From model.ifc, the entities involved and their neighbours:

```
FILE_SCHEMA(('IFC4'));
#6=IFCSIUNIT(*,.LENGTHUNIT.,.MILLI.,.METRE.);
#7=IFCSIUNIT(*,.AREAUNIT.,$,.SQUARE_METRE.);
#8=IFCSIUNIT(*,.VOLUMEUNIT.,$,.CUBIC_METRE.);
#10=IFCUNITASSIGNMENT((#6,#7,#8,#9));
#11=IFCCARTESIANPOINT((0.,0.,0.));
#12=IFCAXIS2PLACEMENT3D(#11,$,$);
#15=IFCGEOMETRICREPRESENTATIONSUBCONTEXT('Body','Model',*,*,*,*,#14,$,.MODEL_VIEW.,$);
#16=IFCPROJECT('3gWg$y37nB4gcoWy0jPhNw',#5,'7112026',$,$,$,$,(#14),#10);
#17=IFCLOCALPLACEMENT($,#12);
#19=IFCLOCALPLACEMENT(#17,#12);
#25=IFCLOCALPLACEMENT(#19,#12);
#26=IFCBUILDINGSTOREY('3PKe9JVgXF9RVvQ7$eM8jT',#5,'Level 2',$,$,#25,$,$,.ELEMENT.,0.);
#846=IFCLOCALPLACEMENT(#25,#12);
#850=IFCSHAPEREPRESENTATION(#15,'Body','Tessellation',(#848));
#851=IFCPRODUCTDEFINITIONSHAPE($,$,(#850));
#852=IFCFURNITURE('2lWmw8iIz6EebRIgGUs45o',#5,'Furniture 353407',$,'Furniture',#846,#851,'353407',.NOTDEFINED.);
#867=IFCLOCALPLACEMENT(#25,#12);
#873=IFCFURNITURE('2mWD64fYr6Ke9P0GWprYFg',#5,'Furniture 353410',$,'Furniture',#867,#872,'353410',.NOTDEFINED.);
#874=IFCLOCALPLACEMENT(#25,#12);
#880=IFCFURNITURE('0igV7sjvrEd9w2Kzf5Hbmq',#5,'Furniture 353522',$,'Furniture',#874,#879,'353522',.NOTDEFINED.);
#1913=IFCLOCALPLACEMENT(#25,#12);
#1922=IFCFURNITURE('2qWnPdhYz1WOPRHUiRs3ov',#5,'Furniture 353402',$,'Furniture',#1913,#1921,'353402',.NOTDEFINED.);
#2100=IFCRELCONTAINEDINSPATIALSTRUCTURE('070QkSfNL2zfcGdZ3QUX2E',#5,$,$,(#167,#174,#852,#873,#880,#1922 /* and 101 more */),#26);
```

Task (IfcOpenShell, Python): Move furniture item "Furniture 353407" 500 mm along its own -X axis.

```python
import ifcopenshell
import ifcopenshell.api.geometry
import ifcopenshell.util.placement
import ifcopenshell.util.unit

model = ifcopenshell.open("model.ifc")
unit_scale = ifcopenshell.util.unit.calculate_unit_scale(model)

item = model.by_guid("2lWmw8iIz6EebRIgGUs45o")
matrix = ifcopenshell.util.placement.get_local_placement(item.ObjectPlacement)
matrix[:3, 3] -= matrix[:3, 0] * 0.5 / unit_scale
ifcopenshell.api.geometry.edit_object_placement(model, product=item, matrix=matrix, is_si=False)

print(ifcopenshell.util.placement.get_local_placement(item.ObjectPlacement).round(3) + 0.0)

model.write("model_v2.ifc")
```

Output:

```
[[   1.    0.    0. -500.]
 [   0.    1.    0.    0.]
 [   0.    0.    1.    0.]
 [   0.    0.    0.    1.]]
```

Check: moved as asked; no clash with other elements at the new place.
